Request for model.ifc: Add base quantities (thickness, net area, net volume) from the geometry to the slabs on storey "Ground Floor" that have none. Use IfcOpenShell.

First a look at what the model holds.

```python
import ifcopenshell
import ifcopenshell.util.element
import ifcopenshell.util.unit

model = ifcopenshell.open("model.ifc")
print(model.schema)
for unit_type in ("LENGTHUNIT", "AREAUNIT", "VOLUMEUNIT"):
    print(unit_type, ifcopenshell.util.unit.calculate_unit_scale(model, unit_type))
storey = next(s for s in model.by_type("IfcBuildingStorey") if s.Name == "Ground Floor")
slabs = [e for e in ifcopenshell.util.element.get_decomposition(storey) if e.is_a("IfcSlab")]
for e in sorted(slabs, key=lambda e: e.id()):
    print(e.id(), e.is_a(), e.Name, list(ifcopenshell.util.element.get_psets(e, qtos_only=True)), sep=" | ")
```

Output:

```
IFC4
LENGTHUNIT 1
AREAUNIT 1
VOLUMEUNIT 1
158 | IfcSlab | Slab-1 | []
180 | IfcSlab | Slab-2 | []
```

```python
import ifcopenshell
import ifcopenshell.api.pset
import ifcopenshell.geom
import ifcopenshell.util.element
import ifcopenshell.util.shape
import ifcopenshell.util.unit

model = ifcopenshell.open("model.ifc")
unit_scale = ifcopenshell.util.unit.calculate_unit_scale(model)
area_scale = ifcopenshell.util.unit.calculate_unit_scale(model, "AREAUNIT")
volume_scale = ifcopenshell.util.unit.calculate_unit_scale(model, "VOLUMEUNIT")
settings = ifcopenshell.geom.settings()

storey = next(s for s in model.by_type("IfcBuildingStorey") if s.Name == "Ground Floor")
slabs = [e for e in ifcopenshell.util.element.get_decomposition(storey) if e.is_a("IfcSlab")]

for e in sorted(slabs, key=lambda e: e.id()):
    if ifcopenshell.util.element.get_psets(e, qtos_only=True, should_inherit=False):
        continue
    # Geometry comes back in metres, in the element's own axes.
    shape = ifcopenshell.geom.create_shape(settings, e)
    values = {
        "Width": ifcopenshell.util.shape.get_z(shape.geometry) / unit_scale,
        "NetArea": ifcopenshell.util.shape.get_footprint_area(shape.geometry) / area_scale,
        "NetVolume": ifcopenshell.util.shape.get_volume(shape.geometry) / volume_scale,
    }
    qto = ifcopenshell.api.pset.add_qto(model, product=e, name="Qto_SlabBaseQuantities")
    ifcopenshell.api.pset.edit_qto(model, qto=qto, properties=values)
    print(e.id(), {k: round(v, 3) for k, v in values.items()})

model.write("model_updated.ifc")
```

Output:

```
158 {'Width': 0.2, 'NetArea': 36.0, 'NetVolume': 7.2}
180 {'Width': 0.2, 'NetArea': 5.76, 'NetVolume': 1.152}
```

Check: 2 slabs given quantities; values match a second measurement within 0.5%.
